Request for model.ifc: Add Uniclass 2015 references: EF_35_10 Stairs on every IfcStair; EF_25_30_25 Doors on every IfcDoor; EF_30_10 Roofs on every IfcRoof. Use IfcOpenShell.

First a look at what the model holds.

```python
import ifcopenshell

model = ifcopenshell.open("model.ifc")
print(model.schema)
print("classifications:", [c.Name for c in model.by_type("IfcClassification")])
for ifc_class in ("IfcDoor", "IfcRoof", "IfcStair", "IfcWall", "IfcWindow"):
    print(ifc_class, len(model.by_type(ifc_class)))
```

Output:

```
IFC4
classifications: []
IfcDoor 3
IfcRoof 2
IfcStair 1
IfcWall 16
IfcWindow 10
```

```python
import ifcopenshell
import ifcopenshell.api.classification

model = ifcopenshell.open("model.ifc")

system = ifcopenshell.api.classification.add_classification(model, classification="Uniclass 2015")

codes = {
    "IfcStair": ("EF_35_10", "Stairs"),
    "IfcDoor": ("EF_25_30_25", "Doors"),
    "IfcRoof": ("EF_30_10", "Roofs"),
}
for ifc_class, (code, name) in codes.items():
    products = model.by_type(ifc_class)
    ifcopenshell.api.classification.add_reference(
        model, products=products, classification=system, identification=code, name=name
    )
    print(code, len(products))

model.write("model_edited.ifc")
```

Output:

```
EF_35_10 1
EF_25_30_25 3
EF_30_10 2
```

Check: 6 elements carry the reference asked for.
